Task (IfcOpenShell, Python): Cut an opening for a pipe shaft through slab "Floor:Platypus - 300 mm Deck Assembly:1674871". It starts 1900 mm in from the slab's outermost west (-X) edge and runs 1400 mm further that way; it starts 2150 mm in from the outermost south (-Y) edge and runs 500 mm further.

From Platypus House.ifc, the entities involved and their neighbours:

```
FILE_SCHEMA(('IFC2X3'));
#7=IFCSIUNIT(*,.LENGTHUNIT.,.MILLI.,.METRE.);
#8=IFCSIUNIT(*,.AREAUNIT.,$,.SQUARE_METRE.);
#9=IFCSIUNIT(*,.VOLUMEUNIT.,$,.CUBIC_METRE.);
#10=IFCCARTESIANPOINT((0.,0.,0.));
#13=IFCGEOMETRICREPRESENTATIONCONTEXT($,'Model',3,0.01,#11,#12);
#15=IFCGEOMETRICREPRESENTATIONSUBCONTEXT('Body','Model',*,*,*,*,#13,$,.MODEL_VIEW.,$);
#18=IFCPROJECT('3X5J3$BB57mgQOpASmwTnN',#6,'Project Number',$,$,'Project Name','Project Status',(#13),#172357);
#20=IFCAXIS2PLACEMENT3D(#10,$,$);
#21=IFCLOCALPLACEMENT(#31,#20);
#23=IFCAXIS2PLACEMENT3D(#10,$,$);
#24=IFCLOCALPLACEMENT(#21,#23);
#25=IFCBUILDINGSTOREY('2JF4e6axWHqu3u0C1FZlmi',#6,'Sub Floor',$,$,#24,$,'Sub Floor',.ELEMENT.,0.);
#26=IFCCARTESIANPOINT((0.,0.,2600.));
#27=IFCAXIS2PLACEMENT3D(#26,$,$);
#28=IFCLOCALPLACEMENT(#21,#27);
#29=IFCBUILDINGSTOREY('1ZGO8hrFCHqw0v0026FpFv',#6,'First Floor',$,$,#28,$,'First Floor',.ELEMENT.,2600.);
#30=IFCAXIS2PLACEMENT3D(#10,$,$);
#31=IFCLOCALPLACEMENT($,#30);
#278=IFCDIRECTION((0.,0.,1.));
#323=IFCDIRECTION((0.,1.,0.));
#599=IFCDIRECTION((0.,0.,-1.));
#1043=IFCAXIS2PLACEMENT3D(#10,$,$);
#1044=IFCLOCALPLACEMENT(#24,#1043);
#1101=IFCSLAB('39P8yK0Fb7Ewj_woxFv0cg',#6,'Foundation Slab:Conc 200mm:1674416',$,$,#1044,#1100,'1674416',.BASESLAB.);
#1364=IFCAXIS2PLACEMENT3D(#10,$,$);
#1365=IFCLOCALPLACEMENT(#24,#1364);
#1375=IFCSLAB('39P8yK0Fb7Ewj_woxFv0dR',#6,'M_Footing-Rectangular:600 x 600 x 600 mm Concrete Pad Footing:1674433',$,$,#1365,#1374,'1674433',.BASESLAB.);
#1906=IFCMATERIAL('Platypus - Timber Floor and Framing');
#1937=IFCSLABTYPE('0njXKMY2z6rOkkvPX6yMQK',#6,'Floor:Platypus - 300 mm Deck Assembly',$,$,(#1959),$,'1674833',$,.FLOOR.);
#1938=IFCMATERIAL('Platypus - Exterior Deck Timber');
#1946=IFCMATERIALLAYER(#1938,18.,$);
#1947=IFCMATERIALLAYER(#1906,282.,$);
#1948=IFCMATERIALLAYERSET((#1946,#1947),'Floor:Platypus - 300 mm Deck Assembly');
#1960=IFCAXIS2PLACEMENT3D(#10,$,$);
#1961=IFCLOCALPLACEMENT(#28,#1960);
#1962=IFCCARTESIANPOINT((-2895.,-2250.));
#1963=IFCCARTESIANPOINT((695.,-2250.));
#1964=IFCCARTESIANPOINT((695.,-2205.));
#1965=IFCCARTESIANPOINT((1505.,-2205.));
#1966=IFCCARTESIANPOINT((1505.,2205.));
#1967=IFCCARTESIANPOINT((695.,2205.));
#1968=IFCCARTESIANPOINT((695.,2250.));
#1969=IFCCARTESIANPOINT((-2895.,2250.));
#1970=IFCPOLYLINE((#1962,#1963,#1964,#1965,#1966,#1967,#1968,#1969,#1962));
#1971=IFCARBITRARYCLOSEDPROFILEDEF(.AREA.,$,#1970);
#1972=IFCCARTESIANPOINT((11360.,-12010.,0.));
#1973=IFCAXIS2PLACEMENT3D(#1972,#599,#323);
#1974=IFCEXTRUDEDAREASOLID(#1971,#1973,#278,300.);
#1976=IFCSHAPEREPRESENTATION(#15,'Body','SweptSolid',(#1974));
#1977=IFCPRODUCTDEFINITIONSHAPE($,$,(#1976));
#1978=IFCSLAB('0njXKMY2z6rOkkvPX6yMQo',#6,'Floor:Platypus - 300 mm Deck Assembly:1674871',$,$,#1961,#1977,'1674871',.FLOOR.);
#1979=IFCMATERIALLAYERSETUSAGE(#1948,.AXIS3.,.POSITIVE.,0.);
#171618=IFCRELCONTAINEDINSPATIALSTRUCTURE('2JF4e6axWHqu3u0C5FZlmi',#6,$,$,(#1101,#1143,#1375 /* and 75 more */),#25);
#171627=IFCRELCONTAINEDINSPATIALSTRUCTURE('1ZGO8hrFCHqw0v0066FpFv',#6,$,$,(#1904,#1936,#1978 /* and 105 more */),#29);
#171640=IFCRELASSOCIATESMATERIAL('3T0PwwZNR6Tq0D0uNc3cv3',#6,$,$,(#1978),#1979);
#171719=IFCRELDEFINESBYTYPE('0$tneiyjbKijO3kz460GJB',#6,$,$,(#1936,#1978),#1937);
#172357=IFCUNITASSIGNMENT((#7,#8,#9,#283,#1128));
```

```python
import numpy as np
import ifcopenshell
import ifcopenshell.api.feature
import ifcopenshell.api.geometry
import ifcopenshell.api.root
import ifcopenshell.geom
import ifcopenshell.util.placement
import ifcopenshell.util.representation
import ifcopenshell.util.shape
import ifcopenshell.util.unit

model = ifcopenshell.open("Platypus House.ifc")
unit_scale = ifcopenshell.util.unit.calculate_unit_scale(model)
settings = ifcopenshell.geom.settings()


def volume(element):
    """Net volume in cubic metres, openings subtracted."""
    shape = ifcopenshell.geom.create_shape(settings, element)
    return ifcopenshell.util.shape.get_volume(shape.geometry)


slab = model.by_id(1978)
before = volume(slab)

# Extent in the slab's own axes, in metres. The edges named are its -X and -Y sides.
slab_shape = ifcopenshell.geom.create_shape(settings, slab)
vertices = ifcopenshell.util.shape.get_vertices(slab_shape.geometry)
x_min, y_min, bottom = vertices.min(axis=0)
top = vertices[:, 2].max()

opening = ifcopenshell.api.root.create_entity(model, ifc_class="IfcOpeningElement", name="Pipe shaft opening")
context = ifcopenshell.util.representation.get_context(model, "Model", "Body", "MODEL_VIEW")
width, depth = 1.4, 0.5
outline = [(0.0, 0.0), (width, 0.0), (width, depth), (0.0, depth), (0.0, 0.0)]
# Overshoot both faces by 50 mm so the cut is clean.
shape = ifcopenshell.api.geometry.add_slab_representation(
    model, context=context, depth=top - bottom + 0.1, polyline=outline
)
ifcopenshell.api.geometry.assign_representation(model, product=opening, representation=shape)

matrix = ifcopenshell.util.placement.get_local_placement(slab.ObjectPlacement)
matrix[:, 3] = matrix @ np.append(np.array([x_min + 1.9, y_min + 2.15, bottom - 0.05]) / unit_scale, 1.0)
ifcopenshell.api.geometry.edit_object_placement(model, product=opening, matrix=matrix, is_si=False)
ifcopenshell.api.feature.add_feature(model, feature=opening, element=slab)

after = volume(slab)

print(f"slab volume {before:.3f} -> {after:.3f} m3")

model.write("Platypus House_v2.ifc")
```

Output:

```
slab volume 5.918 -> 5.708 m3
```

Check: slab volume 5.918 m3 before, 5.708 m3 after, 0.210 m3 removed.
